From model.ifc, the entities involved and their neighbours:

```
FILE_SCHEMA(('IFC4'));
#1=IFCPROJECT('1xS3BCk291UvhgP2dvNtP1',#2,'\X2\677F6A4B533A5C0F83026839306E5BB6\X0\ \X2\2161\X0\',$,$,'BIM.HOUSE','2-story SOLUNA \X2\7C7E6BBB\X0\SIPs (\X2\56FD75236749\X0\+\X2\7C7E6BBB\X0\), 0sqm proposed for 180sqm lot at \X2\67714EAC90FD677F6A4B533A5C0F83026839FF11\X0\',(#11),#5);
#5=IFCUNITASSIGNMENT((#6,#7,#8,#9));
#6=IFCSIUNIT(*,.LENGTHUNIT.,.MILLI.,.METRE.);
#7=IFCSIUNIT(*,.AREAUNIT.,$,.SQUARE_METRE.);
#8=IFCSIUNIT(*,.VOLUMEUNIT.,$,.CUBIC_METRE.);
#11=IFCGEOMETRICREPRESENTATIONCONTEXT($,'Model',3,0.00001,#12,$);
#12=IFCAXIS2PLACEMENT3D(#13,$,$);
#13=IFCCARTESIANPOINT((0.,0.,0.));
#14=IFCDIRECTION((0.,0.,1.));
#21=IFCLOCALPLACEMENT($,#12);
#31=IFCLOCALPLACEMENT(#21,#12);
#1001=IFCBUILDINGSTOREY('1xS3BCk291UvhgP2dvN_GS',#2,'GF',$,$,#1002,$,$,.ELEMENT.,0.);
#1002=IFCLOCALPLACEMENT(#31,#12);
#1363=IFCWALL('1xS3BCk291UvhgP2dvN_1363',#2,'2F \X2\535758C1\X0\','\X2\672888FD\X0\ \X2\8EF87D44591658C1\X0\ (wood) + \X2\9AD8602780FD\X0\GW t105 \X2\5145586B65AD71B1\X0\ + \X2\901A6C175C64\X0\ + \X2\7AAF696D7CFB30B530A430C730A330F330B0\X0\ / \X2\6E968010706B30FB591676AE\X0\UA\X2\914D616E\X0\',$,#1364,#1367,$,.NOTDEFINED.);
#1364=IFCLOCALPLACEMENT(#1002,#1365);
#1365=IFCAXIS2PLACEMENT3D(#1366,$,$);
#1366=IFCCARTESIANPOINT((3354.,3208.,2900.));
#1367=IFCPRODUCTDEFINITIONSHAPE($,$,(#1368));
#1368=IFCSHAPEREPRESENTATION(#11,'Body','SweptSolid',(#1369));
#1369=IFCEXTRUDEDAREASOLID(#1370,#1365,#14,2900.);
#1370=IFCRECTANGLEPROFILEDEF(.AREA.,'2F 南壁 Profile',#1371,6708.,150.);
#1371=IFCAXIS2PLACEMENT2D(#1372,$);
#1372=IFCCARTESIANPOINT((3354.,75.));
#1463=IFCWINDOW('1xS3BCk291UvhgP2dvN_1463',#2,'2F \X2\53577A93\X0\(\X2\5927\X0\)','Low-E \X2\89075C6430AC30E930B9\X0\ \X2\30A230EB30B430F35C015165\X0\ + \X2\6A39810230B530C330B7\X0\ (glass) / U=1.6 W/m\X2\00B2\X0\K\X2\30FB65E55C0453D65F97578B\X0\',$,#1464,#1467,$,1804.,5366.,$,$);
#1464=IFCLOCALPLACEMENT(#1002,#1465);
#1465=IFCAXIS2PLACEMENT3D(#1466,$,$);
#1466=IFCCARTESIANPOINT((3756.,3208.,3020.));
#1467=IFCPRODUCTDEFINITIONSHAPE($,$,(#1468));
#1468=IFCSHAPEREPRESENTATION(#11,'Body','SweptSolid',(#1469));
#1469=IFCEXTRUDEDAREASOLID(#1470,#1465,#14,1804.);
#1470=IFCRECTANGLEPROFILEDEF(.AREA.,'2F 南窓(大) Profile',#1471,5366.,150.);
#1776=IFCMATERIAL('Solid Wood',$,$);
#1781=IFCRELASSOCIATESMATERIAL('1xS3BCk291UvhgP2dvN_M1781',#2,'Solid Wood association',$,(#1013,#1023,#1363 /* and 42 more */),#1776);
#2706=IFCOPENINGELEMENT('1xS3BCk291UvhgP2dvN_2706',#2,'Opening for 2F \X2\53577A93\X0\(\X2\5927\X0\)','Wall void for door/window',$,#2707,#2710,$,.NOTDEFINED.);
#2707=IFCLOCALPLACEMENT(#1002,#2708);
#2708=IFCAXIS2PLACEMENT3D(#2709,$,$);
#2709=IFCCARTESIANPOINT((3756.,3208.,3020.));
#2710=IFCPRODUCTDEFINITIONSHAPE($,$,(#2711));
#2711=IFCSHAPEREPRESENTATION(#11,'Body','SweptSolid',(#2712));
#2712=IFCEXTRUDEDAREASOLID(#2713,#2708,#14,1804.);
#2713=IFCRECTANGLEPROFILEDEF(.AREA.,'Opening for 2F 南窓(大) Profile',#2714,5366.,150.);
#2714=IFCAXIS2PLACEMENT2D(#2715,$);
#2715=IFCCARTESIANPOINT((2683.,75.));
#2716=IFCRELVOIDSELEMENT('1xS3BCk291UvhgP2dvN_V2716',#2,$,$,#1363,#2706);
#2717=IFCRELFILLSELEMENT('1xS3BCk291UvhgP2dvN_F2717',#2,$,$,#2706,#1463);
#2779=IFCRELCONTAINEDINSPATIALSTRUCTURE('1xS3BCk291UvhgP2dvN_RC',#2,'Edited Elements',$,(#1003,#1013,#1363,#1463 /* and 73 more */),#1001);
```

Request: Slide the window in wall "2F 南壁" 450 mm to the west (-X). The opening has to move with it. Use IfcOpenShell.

```python
import ifcopenshell
import ifcopenshell.api.geometry
import ifcopenshell.util.placement

model = ifcopenshell.open("model.ifc")

window = model.by_id(1463)
opening = window.FillsVoids[0].RelatingOpeningElement
wall = opening.VoidsElements[0].RelatingBuildingElement

wall_matrix = ifcopenshell.util.placement.get_local_placement(wall.ObjectPlacement)
shift = wall_matrix[:3, 0] * -450.0
before = ifcopenshell.util.placement.get_local_placement(window.ObjectPlacement)[:3, 3].copy()

# The window is not placed relative to its opening, so move both.
for product in (opening, window):
    matrix = ifcopenshell.util.placement.get_local_placement(product.ObjectPlacement)
    matrix[:3, 3] += shift
    ifcopenshell.api.geometry.edit_object_placement(model, product=product, matrix=matrix, is_si=False)

after = ifcopenshell.util.placement.get_local_placement(window.ObjectPlacement)[:3, 3]
print("window moved by", (after - before).round(3) + 0.0)

model.write("model_edited.ifc")
```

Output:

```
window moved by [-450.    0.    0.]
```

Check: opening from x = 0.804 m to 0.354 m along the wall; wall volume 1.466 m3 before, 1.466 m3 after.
